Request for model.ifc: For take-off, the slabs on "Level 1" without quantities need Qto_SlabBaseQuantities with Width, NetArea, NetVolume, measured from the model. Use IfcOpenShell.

First a look at what the model holds.

```python
import ifcopenshell
import ifcopenshell.util.element
import ifcopenshell.util.unit

model = ifcopenshell.open("model.ifc")
print(model.schema)
for unit_type in ("LENGTHUNIT", "AREAUNIT", "VOLUMEUNIT"):
    print(unit_type, ifcopenshell.util.unit.calculate_unit_scale(model, unit_type))
storey = next(s for s in model.by_type("IfcBuildingStorey") if s.Name == "Level 1")
slabs = [e for e in ifcopenshell.util.element.get_decomposition(storey) if e.is_a("IfcSlab")]
for e in sorted(slabs, key=lambda e: e.id()):
    print(e.id(), e.is_a(), e.Name, list(ifcopenshell.util.element.get_psets(e, qtos_only=True)), sep=" | ")
```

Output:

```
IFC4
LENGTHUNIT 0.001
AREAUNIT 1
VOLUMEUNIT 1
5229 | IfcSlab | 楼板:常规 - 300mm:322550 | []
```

```python
import ifcopenshell
import ifcopenshell.api.pset
import ifcopenshell.geom
import ifcopenshell.util.element
import ifcopenshell.util.shape
import ifcopenshell.util.unit

model = ifcopenshell.open("model.ifc")
unit_scale = ifcopenshell.util.unit.calculate_unit_scale(model)
area_scale = ifcopenshell.util.unit.calculate_unit_scale(model, "AREAUNIT")
volume_scale = ifcopenshell.util.unit.calculate_unit_scale(model, "VOLUMEUNIT")
settings = ifcopenshell.geom.settings()

storey = next(s for s in model.by_type("IfcBuildingStorey") if s.Name == "Level 1")
slabs = [e for e in ifcopenshell.util.element.get_decomposition(storey) if e.is_a("IfcSlab")]

for e in sorted(slabs, key=lambda e: e.id()):
    if ifcopenshell.util.element.get_psets(e, qtos_only=True, should_inherit=False):
        continue
    # Geometry comes back in metres, in the element's own axes.
    shape = ifcopenshell.geom.create_shape(settings, e)
    values = {
        "Width": ifcopenshell.util.shape.get_z(shape.geometry) / unit_scale,
        "NetArea": ifcopenshell.util.shape.get_footprint_area(shape.geometry) / area_scale,
        "NetVolume": ifcopenshell.util.shape.get_volume(shape.geometry) / volume_scale,
    }
    qto = ifcopenshell.api.pset.add_qto(model, product=e, name="Qto_SlabBaseQuantities")
    ifcopenshell.api.pset.edit_qto(model, qto=qto, properties=values)
    print(e.id(), {k: round(v, 3) for k, v in values.items()})

model.write("model_updated.ifc")
```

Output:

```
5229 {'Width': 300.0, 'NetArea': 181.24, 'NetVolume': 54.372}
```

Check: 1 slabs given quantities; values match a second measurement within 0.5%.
